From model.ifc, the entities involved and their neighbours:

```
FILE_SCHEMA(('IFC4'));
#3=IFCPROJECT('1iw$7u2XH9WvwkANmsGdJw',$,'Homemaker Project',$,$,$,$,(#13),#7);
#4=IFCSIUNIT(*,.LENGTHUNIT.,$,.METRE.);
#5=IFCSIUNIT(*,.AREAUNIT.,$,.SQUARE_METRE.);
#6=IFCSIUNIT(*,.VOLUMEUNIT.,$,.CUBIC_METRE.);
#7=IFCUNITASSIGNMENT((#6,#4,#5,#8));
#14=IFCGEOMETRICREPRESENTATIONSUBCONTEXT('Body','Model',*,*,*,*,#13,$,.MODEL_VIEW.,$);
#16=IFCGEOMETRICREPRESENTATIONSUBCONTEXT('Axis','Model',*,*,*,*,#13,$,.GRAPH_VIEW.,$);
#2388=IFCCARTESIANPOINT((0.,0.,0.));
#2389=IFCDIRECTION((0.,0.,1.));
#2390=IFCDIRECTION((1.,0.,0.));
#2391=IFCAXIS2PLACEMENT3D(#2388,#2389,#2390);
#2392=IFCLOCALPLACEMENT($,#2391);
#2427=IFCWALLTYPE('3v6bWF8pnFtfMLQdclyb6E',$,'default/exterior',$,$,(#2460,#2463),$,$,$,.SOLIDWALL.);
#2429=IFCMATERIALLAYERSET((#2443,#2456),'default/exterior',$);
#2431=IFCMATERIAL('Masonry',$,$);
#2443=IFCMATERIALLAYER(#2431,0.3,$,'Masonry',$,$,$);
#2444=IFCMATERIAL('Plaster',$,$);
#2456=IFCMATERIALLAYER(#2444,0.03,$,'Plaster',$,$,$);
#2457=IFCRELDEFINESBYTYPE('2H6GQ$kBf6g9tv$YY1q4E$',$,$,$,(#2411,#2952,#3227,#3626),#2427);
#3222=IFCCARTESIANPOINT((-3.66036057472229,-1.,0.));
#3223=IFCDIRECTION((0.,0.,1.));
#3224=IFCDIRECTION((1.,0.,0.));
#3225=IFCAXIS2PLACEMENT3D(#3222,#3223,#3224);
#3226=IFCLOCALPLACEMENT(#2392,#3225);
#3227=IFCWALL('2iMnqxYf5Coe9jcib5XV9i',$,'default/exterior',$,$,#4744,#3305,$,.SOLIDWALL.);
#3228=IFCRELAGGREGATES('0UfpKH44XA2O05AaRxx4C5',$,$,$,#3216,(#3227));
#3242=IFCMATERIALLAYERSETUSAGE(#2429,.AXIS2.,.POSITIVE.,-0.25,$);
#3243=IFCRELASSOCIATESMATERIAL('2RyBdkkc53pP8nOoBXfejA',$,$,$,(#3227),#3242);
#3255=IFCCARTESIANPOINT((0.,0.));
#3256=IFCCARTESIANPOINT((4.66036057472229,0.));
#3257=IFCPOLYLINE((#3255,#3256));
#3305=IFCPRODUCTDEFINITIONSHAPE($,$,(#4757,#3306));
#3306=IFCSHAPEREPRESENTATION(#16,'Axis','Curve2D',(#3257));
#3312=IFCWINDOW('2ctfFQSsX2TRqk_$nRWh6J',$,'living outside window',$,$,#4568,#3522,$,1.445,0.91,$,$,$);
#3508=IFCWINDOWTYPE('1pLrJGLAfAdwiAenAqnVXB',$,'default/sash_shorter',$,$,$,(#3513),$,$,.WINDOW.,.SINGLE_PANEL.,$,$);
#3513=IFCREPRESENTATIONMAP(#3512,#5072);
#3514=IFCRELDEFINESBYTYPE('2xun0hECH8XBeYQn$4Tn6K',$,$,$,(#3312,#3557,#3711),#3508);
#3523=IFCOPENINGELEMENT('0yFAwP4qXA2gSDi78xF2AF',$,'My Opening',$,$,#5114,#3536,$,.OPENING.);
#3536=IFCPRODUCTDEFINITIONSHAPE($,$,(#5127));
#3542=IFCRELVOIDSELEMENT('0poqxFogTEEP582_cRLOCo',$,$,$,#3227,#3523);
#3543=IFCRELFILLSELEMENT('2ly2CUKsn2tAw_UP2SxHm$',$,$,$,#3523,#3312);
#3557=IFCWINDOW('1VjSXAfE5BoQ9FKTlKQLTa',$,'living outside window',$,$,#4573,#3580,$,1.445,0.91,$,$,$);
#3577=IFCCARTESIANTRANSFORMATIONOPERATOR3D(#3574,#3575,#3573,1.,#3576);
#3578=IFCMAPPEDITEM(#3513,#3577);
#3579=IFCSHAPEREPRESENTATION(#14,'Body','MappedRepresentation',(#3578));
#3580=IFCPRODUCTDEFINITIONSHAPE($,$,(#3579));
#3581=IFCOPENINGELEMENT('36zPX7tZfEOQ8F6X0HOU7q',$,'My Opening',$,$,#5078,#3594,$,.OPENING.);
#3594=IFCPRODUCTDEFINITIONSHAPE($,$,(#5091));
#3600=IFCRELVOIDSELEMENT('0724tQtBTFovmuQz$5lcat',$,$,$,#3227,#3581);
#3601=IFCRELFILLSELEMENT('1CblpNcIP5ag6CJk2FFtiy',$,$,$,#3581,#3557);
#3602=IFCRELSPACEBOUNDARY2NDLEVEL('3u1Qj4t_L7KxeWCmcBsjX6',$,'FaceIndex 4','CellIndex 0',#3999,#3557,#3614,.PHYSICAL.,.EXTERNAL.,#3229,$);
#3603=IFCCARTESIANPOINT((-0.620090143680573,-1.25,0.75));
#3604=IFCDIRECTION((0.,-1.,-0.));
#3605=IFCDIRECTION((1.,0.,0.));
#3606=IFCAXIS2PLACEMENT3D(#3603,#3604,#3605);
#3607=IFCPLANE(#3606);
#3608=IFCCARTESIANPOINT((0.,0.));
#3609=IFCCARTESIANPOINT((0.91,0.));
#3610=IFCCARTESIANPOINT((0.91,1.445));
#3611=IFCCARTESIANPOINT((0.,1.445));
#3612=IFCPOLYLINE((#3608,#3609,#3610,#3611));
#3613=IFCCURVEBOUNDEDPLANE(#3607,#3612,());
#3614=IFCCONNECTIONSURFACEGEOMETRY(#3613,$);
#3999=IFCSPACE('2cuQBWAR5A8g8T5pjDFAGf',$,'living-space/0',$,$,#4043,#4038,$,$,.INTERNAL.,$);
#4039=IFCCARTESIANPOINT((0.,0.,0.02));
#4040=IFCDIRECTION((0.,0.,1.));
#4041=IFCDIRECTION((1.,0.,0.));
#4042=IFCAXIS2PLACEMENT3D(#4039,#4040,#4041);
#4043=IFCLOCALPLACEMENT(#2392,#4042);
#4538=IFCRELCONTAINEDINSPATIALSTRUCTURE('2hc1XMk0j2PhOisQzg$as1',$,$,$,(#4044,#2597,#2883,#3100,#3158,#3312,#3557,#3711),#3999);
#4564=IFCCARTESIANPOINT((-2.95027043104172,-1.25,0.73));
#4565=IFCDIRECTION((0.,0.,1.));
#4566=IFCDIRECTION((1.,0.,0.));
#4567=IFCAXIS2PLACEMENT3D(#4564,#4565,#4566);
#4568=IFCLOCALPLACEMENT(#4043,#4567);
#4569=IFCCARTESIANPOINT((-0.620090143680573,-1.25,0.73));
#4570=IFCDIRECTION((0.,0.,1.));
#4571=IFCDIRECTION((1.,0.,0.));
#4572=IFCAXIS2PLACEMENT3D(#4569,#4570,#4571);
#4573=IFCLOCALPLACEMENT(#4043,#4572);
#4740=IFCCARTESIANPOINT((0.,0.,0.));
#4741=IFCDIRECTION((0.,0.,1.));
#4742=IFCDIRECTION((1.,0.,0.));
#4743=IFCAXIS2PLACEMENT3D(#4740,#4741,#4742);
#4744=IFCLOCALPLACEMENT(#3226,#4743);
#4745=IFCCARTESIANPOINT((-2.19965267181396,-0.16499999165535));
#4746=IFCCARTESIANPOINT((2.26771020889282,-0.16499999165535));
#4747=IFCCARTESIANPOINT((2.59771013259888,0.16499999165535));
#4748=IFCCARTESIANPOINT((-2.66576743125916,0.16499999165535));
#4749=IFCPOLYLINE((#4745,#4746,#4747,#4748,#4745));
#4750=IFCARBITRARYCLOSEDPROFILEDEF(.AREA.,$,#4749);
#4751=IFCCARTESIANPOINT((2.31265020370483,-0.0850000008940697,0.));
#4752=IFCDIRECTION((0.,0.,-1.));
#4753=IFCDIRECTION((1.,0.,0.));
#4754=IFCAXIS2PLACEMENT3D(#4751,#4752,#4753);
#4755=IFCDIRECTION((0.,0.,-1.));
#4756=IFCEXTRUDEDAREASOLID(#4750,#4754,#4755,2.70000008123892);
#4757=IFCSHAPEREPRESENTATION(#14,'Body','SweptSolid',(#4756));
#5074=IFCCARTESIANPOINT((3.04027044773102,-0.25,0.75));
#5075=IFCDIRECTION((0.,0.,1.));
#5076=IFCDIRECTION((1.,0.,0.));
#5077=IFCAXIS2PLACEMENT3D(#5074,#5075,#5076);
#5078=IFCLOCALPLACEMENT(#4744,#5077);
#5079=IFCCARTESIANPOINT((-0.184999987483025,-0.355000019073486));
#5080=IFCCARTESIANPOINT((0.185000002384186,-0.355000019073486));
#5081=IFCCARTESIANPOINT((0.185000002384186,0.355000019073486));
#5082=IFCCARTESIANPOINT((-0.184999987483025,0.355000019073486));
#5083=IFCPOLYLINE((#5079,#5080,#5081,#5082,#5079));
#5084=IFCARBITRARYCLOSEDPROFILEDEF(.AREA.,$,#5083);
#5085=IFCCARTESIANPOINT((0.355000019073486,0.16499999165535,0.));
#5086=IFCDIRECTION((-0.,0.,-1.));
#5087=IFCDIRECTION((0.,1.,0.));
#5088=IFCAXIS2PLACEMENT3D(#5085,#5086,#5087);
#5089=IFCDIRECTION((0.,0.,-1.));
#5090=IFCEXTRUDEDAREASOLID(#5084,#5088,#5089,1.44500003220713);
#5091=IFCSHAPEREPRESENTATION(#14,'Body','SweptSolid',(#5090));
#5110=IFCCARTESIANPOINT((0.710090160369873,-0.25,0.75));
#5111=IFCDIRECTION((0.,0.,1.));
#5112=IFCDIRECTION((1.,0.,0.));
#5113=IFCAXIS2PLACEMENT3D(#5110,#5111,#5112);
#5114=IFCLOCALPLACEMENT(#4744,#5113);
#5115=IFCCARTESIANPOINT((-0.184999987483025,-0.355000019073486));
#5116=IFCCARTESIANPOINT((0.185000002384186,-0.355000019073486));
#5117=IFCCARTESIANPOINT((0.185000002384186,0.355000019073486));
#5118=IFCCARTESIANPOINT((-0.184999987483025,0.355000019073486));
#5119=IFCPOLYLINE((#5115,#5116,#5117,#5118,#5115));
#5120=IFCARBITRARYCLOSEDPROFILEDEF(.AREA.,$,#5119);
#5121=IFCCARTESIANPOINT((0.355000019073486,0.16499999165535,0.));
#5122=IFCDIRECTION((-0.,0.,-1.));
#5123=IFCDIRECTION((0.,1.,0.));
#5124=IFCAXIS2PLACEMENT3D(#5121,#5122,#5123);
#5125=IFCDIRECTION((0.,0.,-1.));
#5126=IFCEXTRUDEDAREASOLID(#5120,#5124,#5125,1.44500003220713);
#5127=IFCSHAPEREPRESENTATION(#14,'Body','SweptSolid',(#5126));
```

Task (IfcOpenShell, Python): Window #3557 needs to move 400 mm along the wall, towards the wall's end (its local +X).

```python
import numpy as np
import ifcopenshell
import ifcopenshell.api.geometry
import ifcopenshell.util.placement

model = ifcopenshell.open("model.ifc")

window = model.by_guid("1VjSXAfE5BoQ9FKTlKQLTa")
opening = window.FillsVoids[0].RelatingOpeningElement
wall = opening.VoidsElements[0].RelatingBuildingElement

wall_matrix = ifcopenshell.util.placement.get_local_placement(wall.ObjectPlacement)
shift = wall_matrix[:3, 0] * 0.4
before = ifcopenshell.util.placement.get_local_placement(window.ObjectPlacement)[:3, 3].copy()

# The window is not placed relative to its opening, so move both.
for product in (opening, window):
    matrix = ifcopenshell.util.placement.get_local_placement(product.ObjectPlacement)
    matrix[:3, 3] += shift
    ifcopenshell.api.geometry.edit_object_placement(model, product=product, matrix=matrix, is_si=False)

# Space boundary surfaces are stored in each space's coordinates; move them too.
for rel in window.ProvidesBoundaries:
    if not rel.ConnectionGeometry:
        continue
    surface = rel.ConnectionGeometry.SurfaceOnRelatingElement.BasisSurface
    space_matrix = ifcopenshell.util.placement.get_local_placement(rel.RelatingSpace.ObjectPlacement)
    point = np.array(surface.Position.Location.Coordinates) + space_matrix[:3, :3].T @ shift
    surface.Position = model.createIfcAxis2Placement3D(
        model.createIfcCartesianPoint(point.tolist()), surface.Position.Axis, surface.Position.RefDirection
    )

after = ifcopenshell.util.placement.get_local_placement(window.ObjectPlacement)[:3, 3]
print("window moved by", (after - before).round(3) + 0.0)

model.write("model-out.ifc")
```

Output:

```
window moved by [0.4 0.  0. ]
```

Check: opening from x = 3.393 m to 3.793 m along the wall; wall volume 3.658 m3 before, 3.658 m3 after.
